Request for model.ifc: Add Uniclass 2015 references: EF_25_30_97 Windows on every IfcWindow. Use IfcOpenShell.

First a look at what the model holds.

```python
import ifcopenshell

model = ifcopenshell.open("model.ifc")
print(model.schema)
print("classifications:", [c.Name for c in model.by_type("IfcClassification")])
for ifc_class in ("IfcDoor", "IfcRoof", "IfcStair", "IfcWall", "IfcWindow"):
    print(ifc_class, len(model.by_type(ifc_class)))
```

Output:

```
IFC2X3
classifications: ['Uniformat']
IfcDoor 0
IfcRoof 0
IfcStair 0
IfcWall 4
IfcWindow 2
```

```python
import ifcopenshell
import ifcopenshell.api.classification

model = ifcopenshell.open("model.ifc")

# IFC2X3 requires Source and Edition and has no link from the project to the system.
system = model.create_entity("IfcClassification", Source="NBS", Edition="2015", Name="Uniclass 2015")

codes = {
    "IfcWindow": ("EF_25_30_97", "Windows"),
}
for ifc_class, (code, name) in codes.items():
    products = model.by_type(ifc_class)
    ifcopenshell.api.classification.add_reference(
        model, products=products, classification=system, identification=code, name=name
    )
    print(code, len(products))

model.write("model_v2.ifc")
```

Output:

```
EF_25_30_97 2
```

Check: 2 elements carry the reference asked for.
